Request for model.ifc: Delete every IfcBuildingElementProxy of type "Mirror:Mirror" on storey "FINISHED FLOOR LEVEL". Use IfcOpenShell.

First a look at what the model holds.

```python
import ifcopenshell
import ifcopenshell.util.element

model = ifcopenshell.open("model.ifc")
print(model.schema)
storey = next(s for s in model.by_type("IfcBuildingStorey") if s.Name == "FINISHED FLOOR LEVEL")
proxies = [e for e in ifcopenshell.util.element.get_decomposition(storey) if e.is_a("IfcBuildingElementProxy")]
seen = {}
for e in proxies:
    element_type = ifcopenshell.util.element.get_type(e)
    name = element_type.Name if element_type not in (None, e) else None
    seen[name] = seen.get(name, 0) + 1
for name, count in sorted(seen.items(), key=str):
    print(count, "x", name)
```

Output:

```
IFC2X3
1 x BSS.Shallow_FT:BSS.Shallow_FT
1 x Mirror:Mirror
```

```python
import ifcopenshell
import ifcopenshell.api.root
import ifcopenshell.util.element

model = ifcopenshell.open("model.ifc")

storey = next(s for s in model.by_type("IfcBuildingStorey") if s.Name == "FINISHED FLOOR LEVEL")
proxies = [e for e in ifcopenshell.util.element.get_decomposition(storey) if e.is_a("IfcBuildingElementProxy")]
targets = [e for e in proxies if (t := ifcopenshell.util.element.get_type(e)) not in (None, e) and t.Name == "Mirror:Mirror"]

for e in targets:
    ifcopenshell.api.root.remove_product(model, product=e)
print(len(targets), "removed")

model.write("model_v2.ifc")
```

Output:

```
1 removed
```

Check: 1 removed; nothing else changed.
